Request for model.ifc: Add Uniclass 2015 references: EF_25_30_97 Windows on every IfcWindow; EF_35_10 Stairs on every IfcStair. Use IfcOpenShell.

First a look at what the model holds.

```python
import ifcopenshell

model = ifcopenshell.open("model.ifc")
print(model.schema)
print("classifications:", [c.Name for c in model.by_type("IfcClassification")])
for ifc_class in ("IfcDoor", "IfcRoof", "IfcStair", "IfcWall", "IfcWindow"):
    print(ifc_class, len(model.by_type(ifc_class)))
```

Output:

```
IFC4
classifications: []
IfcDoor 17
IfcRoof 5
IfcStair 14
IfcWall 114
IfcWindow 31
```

```python
import ifcopenshell
import ifcopenshell.api.classification

model = ifcopenshell.open("model.ifc")

system = ifcopenshell.api.classification.add_classification(model, classification="Uniclass 2015")

codes = {
    "IfcWindow": ("EF_25_30_97", "Windows"),
    "IfcStair": ("EF_35_10", "Stairs"),
}
for ifc_class, (code, name) in codes.items():
    products = model.by_type(ifc_class)
    ifcopenshell.api.classification.add_reference(
        model, products=products, classification=system, identification=code, name=name
    )
    print(code, len(products))

model.write("model-out.ifc")
```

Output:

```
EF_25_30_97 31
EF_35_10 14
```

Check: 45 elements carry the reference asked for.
